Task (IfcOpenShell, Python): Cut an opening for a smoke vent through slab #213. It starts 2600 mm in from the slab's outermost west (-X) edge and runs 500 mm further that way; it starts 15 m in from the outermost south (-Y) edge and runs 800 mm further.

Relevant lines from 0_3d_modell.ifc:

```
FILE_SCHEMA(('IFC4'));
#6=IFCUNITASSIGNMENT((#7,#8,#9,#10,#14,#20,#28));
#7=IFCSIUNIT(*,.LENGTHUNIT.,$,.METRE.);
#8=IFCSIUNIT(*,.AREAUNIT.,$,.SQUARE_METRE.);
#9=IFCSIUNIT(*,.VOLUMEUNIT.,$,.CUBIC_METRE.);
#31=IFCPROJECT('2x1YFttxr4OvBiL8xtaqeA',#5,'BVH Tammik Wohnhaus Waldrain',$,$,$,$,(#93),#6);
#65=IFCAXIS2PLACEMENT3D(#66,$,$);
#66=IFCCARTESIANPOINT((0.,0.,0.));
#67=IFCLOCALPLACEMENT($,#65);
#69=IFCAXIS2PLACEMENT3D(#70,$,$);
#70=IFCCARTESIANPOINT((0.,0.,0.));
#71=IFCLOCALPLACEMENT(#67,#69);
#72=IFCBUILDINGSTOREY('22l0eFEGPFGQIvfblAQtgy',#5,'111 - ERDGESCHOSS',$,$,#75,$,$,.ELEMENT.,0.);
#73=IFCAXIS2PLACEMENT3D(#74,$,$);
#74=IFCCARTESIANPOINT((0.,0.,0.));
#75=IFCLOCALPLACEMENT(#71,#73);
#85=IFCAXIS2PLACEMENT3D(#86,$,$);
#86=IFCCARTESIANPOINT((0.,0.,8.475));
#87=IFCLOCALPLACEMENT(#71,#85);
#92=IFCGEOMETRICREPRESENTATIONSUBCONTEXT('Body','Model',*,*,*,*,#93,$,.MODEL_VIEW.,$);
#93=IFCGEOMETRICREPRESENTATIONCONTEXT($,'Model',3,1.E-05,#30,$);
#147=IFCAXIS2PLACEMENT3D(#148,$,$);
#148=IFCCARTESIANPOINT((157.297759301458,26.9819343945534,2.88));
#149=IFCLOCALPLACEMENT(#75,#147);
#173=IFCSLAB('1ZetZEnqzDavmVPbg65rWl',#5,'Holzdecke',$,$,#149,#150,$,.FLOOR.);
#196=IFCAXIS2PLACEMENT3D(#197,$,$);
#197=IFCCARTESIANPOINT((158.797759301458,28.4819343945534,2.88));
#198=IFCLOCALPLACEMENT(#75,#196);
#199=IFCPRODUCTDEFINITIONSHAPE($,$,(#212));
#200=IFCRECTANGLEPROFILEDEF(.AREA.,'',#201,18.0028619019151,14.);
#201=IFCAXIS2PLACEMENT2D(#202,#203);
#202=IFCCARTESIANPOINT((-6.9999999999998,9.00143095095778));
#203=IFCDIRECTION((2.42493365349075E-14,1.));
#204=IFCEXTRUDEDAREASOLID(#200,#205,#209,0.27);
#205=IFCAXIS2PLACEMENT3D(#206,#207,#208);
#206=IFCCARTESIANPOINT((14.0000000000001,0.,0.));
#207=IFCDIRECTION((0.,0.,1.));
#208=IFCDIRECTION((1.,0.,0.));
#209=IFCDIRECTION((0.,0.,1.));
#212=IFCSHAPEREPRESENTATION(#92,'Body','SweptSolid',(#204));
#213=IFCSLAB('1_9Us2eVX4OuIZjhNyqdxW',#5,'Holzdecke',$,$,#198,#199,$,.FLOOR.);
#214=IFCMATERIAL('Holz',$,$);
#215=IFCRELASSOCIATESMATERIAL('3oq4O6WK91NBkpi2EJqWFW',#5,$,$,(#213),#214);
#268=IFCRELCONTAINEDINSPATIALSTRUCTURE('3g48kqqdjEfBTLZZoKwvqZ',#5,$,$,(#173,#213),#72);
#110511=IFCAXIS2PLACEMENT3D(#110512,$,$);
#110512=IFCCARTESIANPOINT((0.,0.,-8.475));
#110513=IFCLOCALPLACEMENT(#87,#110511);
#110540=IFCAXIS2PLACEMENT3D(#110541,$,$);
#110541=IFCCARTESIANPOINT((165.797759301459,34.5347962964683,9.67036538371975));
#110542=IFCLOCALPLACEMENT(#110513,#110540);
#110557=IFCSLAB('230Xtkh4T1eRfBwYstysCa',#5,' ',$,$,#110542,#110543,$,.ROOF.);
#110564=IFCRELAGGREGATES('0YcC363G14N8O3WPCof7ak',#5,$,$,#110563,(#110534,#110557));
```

```python
import numpy as np
import ifcopenshell
import ifcopenshell.api.feature
import ifcopenshell.api.geometry
import ifcopenshell.api.root
import ifcopenshell.geom
import ifcopenshell.util.placement
import ifcopenshell.util.representation
import ifcopenshell.util.shape
import ifcopenshell.util.unit

model = ifcopenshell.open("0_3d_modell.ifc")
unit_scale = ifcopenshell.util.unit.calculate_unit_scale(model)
settings = ifcopenshell.geom.settings()


def volume(element):
    """Net volume in cubic metres, openings subtracted."""
    shape = ifcopenshell.geom.create_shape(settings, element)
    return ifcopenshell.util.shape.get_volume(shape.geometry)


slab = model.by_id(213)
before = volume(slab)

# Extent in the slab's own axes, in metres. The edges named are its -X and -Y sides.
slab_shape = ifcopenshell.geom.create_shape(settings, slab)
vertices = ifcopenshell.util.shape.get_vertices(slab_shape.geometry)
x_min, y_min, bottom = vertices.min(axis=0)
top = vertices[:, 2].max()

opening = ifcopenshell.api.root.create_entity(model, ifc_class="IfcOpeningElement", name="Smoke vent opening", predefined_type="OPENING")
context = ifcopenshell.util.representation.get_context(model, "Model", "Body", "MODEL_VIEW")
width, depth = 0.5, 0.8
outline = [(0.0, 0.0), (width, 0.0), (width, depth), (0.0, depth), (0.0, 0.0)]
# Overshoot both faces by 50 mm so the cut is clean.
shape = ifcopenshell.api.geometry.add_slab_representation(
    model, context=context, depth=top - bottom + 0.1, polyline=outline
)
ifcopenshell.api.geometry.assign_representation(model, product=opening, representation=shape)

matrix = ifcopenshell.util.placement.get_local_placement(slab.ObjectPlacement)
matrix[:, 3] = matrix @ np.append(np.array([x_min + 2.6, y_min + 15, bottom - 0.05]) / unit_scale, 1.0)
ifcopenshell.api.geometry.edit_object_placement(model, product=opening, matrix=matrix, is_si=False)
ifcopenshell.api.feature.add_feature(model, feature=opening, element=slab)

after = volume(slab)

print(f"slab volume {before:.3f} -> {after:.3f} m3")

model.write("0_3d_modell_v2.ifc")
```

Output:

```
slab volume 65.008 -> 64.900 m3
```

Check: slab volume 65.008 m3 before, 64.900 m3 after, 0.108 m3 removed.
